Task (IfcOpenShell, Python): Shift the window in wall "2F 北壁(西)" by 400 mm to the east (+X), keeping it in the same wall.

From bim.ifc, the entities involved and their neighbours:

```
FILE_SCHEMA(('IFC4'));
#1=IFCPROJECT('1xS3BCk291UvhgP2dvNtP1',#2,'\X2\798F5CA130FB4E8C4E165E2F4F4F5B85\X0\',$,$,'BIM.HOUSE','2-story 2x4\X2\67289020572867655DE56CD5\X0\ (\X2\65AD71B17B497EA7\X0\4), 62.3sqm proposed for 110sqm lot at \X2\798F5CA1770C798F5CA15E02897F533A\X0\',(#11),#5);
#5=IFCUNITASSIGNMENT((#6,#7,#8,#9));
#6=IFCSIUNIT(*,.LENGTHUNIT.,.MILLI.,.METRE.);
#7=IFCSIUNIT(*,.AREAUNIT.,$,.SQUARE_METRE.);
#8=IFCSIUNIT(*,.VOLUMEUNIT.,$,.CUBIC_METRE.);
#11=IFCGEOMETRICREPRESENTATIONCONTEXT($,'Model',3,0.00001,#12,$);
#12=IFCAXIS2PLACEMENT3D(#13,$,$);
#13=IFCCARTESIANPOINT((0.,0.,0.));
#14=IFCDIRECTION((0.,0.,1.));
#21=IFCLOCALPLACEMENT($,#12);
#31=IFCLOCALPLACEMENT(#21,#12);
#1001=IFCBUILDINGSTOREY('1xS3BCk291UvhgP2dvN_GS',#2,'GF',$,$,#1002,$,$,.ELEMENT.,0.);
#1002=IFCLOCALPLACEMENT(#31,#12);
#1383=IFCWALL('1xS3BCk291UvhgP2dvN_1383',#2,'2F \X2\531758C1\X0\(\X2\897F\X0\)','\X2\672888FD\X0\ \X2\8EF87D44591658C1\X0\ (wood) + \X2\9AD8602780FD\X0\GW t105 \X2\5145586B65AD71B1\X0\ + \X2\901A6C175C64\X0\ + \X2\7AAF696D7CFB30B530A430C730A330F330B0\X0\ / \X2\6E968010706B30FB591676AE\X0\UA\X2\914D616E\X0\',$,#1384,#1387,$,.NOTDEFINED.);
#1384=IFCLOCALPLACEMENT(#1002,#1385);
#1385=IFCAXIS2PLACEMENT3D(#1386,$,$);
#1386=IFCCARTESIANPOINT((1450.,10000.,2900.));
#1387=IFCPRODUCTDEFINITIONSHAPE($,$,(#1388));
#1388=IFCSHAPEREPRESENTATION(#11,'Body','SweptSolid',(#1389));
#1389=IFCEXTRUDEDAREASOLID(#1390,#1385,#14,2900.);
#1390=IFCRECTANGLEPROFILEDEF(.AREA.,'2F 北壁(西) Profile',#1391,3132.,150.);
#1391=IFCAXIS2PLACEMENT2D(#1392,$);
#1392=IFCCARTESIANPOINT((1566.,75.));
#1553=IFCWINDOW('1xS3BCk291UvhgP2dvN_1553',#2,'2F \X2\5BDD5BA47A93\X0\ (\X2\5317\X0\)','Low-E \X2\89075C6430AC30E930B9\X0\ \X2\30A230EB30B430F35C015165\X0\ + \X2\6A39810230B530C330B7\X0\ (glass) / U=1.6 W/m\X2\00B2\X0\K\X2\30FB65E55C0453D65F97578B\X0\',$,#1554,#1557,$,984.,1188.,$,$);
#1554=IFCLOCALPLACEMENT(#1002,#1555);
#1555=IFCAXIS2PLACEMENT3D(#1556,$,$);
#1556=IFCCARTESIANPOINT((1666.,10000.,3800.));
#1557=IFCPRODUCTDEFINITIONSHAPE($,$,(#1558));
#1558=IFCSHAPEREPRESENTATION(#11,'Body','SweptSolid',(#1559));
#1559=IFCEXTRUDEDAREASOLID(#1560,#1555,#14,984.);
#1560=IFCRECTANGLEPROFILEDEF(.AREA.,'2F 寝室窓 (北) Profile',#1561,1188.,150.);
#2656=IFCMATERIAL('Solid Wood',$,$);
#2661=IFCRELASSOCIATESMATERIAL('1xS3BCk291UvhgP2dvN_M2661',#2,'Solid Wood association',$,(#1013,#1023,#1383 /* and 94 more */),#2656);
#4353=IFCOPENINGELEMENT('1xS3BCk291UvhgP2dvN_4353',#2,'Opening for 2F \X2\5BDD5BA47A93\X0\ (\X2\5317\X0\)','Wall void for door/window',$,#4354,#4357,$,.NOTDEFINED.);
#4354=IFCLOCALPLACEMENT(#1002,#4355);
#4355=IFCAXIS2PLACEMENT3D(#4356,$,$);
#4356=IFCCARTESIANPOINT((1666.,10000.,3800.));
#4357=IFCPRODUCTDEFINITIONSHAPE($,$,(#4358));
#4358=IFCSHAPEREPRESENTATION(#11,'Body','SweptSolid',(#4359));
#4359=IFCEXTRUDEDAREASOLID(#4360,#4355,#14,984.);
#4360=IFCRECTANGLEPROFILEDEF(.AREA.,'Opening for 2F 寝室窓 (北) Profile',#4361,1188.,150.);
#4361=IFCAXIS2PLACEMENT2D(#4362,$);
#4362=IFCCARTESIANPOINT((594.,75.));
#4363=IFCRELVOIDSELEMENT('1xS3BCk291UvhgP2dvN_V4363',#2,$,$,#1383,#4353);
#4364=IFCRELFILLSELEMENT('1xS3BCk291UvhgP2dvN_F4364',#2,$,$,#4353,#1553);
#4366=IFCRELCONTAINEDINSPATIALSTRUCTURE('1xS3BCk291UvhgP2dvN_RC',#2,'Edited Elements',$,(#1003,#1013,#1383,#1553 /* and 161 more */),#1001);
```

```python
import ifcopenshell
import ifcopenshell.api.geometry
import ifcopenshell.util.placement
import ifcopenshell.util.unit

model = ifcopenshell.open("bim.ifc")
unit_scale = ifcopenshell.util.unit.calculate_unit_scale(model)

window = model.by_guid("1xS3BCk291UvhgP2dvN_1553")
opening = window.FillsVoids[0].RelatingOpeningElement
wall = opening.VoidsElements[0].RelatingBuildingElement

wall_matrix = ifcopenshell.util.placement.get_local_placement(wall.ObjectPlacement)
shift = wall_matrix[:3, 0] * 0.4 / unit_scale
before = ifcopenshell.util.placement.get_local_placement(window.ObjectPlacement)[:3, 3].copy()

# The window is not placed relative to its opening, so move both.
for product in (opening, window):
    matrix = ifcopenshell.util.placement.get_local_placement(product.ObjectPlacement)
    matrix[:3, 3] += shift
    ifcopenshell.api.geometry.edit_object_placement(model, product=product, matrix=matrix, is_si=False)

after = ifcopenshell.util.placement.get_local_placement(window.ObjectPlacement)[:3, 3]
print("window moved by", (after - before).round(3) + 0.0)

model.write("bim_rev.ifc")
```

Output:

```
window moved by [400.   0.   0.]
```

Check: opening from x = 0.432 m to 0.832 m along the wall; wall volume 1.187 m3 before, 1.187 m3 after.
